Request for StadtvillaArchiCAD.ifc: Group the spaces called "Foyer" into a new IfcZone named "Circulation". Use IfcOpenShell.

First a look at what the model holds.

```python
import ifcopenshell

model = ifcopenshell.open("StadtvillaArchiCAD.ifc")
print(model.schema)
seen = {}
for space in model.by_type("IfcSpace"):
    seen[space.LongName] = seen.get(space.LongName, 0) + 1
for name, count in sorted(seen.items(), key=str):
    print(count, "x", name)
print("zones:", [z.Name for z in model.by_type("IfcZone")][:20])
```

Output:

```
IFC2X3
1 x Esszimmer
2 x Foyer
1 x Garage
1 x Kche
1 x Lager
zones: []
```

```python
import ifcopenshell
import ifcopenshell.api.group
import ifcopenshell.api.root

model = ifcopenshell.open("StadtvillaArchiCAD.ifc")

names = {"Foyer"}
spaces = [s for s in model.by_type("IfcSpace") if s.LongName in names]

zone = ifcopenshell.api.root.create_entity(model, ifc_class="IfcZone", name="Circulation")
ifcopenshell.api.group.assign_group(model, products=spaces, group=zone)
print(len(spaces), "spaces in", zone.Name)

model.write("StadtvillaArchiCAD_edited.ifc")
```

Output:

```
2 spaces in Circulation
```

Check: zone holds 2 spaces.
